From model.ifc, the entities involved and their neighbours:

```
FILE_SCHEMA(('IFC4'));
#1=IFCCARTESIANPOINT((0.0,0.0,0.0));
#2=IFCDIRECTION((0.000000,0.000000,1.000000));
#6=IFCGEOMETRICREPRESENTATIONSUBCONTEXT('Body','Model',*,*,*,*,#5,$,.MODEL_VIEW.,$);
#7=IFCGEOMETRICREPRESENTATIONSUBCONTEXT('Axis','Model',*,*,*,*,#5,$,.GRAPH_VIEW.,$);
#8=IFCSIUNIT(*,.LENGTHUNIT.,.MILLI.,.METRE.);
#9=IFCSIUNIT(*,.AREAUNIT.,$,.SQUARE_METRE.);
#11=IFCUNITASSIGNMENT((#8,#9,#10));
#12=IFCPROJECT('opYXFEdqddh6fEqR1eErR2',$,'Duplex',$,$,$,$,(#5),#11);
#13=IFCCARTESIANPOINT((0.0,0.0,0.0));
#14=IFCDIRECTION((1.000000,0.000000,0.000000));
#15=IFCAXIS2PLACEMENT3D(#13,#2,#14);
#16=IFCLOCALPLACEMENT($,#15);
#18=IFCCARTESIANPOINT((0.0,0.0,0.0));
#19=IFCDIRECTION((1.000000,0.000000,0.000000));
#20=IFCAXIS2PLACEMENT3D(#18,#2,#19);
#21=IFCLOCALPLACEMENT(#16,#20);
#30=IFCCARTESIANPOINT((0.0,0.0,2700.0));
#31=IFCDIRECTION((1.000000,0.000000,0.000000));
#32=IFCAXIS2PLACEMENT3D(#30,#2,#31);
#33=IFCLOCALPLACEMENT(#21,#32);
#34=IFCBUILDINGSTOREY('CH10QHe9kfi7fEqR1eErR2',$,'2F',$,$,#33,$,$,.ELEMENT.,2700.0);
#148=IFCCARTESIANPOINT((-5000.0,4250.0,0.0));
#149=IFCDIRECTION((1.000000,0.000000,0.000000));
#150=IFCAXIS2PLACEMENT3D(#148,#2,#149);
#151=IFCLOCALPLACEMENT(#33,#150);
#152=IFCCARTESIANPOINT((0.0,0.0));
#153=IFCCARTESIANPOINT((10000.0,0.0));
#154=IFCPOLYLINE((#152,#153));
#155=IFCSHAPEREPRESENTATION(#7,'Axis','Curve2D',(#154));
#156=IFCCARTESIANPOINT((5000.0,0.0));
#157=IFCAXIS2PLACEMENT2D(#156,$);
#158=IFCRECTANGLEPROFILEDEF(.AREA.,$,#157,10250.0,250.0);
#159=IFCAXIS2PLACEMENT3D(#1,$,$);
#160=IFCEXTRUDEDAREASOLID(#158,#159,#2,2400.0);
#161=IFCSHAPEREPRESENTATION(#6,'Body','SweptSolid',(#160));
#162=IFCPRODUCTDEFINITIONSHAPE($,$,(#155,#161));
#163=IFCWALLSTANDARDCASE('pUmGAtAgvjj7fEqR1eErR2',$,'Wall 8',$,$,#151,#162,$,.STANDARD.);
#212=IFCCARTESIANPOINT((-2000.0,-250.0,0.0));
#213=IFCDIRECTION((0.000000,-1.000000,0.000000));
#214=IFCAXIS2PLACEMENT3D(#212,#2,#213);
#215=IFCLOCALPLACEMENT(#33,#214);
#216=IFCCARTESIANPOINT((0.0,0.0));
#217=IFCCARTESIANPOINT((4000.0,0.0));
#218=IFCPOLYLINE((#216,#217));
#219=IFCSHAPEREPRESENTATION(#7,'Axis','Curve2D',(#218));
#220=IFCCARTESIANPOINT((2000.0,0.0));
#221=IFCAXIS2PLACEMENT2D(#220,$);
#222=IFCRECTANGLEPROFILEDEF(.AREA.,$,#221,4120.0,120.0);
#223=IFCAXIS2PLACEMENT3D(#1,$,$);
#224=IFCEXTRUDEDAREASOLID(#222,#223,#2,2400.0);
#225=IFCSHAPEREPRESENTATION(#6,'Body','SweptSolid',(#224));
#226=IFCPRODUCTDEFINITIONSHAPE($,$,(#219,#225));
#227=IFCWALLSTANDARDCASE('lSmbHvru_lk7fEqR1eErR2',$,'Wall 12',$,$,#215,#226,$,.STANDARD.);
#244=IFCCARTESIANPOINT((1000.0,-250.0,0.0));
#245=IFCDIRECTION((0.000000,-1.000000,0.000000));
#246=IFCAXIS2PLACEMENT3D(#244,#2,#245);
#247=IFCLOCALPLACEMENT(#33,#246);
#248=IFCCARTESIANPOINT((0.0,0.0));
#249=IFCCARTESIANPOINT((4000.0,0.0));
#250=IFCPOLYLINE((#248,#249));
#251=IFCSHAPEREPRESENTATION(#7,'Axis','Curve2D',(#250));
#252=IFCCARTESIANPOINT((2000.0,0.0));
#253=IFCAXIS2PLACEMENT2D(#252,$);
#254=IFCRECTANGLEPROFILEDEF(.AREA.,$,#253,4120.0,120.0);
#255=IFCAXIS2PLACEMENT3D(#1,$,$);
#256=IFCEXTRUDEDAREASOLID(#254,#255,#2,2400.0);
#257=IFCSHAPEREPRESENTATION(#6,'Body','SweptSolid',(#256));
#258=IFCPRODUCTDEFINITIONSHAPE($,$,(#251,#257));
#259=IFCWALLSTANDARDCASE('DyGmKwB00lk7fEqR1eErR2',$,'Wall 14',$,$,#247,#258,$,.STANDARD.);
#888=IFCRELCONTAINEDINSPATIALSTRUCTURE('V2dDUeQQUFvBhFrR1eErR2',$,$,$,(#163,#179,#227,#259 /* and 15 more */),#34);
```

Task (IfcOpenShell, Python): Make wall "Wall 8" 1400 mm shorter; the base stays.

```python
import ifcopenshell
import ifcopenshell.geom
import ifcopenshell.util.representation
import ifcopenshell.util.shape
import ifcopenshell.util.unit

model = ifcopenshell.open("model.ifc")
unit_scale = ifcopenshell.util.unit.calculate_unit_scale(model)
settings = ifcopenshell.geom.settings()


def volume(element):
    """Net volume in cubic metres, openings subtracted."""
    shape = ifcopenshell.geom.create_shape(settings, element)
    return ifcopenshell.util.shape.get_volume(shape.geometry)


wall = model.by_guid("pUmGAtAgvjj7fEqR1eErR2")
before = volume(wall)

body = ifcopenshell.util.representation.get_representation(wall, "Model", "Body")
solid = body.Items[0]
old_height = solid.Depth
solid.Depth -= 1.4 / unit_scale
after = volume(wall)

print(f"height {old_height:g} -> {solid.Depth:g}, volume {before:.3f} -> {after:.3f} m3")

model.write("model_v2.ifc")
```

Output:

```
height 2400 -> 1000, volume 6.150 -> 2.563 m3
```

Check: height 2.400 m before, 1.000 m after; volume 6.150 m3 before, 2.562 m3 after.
